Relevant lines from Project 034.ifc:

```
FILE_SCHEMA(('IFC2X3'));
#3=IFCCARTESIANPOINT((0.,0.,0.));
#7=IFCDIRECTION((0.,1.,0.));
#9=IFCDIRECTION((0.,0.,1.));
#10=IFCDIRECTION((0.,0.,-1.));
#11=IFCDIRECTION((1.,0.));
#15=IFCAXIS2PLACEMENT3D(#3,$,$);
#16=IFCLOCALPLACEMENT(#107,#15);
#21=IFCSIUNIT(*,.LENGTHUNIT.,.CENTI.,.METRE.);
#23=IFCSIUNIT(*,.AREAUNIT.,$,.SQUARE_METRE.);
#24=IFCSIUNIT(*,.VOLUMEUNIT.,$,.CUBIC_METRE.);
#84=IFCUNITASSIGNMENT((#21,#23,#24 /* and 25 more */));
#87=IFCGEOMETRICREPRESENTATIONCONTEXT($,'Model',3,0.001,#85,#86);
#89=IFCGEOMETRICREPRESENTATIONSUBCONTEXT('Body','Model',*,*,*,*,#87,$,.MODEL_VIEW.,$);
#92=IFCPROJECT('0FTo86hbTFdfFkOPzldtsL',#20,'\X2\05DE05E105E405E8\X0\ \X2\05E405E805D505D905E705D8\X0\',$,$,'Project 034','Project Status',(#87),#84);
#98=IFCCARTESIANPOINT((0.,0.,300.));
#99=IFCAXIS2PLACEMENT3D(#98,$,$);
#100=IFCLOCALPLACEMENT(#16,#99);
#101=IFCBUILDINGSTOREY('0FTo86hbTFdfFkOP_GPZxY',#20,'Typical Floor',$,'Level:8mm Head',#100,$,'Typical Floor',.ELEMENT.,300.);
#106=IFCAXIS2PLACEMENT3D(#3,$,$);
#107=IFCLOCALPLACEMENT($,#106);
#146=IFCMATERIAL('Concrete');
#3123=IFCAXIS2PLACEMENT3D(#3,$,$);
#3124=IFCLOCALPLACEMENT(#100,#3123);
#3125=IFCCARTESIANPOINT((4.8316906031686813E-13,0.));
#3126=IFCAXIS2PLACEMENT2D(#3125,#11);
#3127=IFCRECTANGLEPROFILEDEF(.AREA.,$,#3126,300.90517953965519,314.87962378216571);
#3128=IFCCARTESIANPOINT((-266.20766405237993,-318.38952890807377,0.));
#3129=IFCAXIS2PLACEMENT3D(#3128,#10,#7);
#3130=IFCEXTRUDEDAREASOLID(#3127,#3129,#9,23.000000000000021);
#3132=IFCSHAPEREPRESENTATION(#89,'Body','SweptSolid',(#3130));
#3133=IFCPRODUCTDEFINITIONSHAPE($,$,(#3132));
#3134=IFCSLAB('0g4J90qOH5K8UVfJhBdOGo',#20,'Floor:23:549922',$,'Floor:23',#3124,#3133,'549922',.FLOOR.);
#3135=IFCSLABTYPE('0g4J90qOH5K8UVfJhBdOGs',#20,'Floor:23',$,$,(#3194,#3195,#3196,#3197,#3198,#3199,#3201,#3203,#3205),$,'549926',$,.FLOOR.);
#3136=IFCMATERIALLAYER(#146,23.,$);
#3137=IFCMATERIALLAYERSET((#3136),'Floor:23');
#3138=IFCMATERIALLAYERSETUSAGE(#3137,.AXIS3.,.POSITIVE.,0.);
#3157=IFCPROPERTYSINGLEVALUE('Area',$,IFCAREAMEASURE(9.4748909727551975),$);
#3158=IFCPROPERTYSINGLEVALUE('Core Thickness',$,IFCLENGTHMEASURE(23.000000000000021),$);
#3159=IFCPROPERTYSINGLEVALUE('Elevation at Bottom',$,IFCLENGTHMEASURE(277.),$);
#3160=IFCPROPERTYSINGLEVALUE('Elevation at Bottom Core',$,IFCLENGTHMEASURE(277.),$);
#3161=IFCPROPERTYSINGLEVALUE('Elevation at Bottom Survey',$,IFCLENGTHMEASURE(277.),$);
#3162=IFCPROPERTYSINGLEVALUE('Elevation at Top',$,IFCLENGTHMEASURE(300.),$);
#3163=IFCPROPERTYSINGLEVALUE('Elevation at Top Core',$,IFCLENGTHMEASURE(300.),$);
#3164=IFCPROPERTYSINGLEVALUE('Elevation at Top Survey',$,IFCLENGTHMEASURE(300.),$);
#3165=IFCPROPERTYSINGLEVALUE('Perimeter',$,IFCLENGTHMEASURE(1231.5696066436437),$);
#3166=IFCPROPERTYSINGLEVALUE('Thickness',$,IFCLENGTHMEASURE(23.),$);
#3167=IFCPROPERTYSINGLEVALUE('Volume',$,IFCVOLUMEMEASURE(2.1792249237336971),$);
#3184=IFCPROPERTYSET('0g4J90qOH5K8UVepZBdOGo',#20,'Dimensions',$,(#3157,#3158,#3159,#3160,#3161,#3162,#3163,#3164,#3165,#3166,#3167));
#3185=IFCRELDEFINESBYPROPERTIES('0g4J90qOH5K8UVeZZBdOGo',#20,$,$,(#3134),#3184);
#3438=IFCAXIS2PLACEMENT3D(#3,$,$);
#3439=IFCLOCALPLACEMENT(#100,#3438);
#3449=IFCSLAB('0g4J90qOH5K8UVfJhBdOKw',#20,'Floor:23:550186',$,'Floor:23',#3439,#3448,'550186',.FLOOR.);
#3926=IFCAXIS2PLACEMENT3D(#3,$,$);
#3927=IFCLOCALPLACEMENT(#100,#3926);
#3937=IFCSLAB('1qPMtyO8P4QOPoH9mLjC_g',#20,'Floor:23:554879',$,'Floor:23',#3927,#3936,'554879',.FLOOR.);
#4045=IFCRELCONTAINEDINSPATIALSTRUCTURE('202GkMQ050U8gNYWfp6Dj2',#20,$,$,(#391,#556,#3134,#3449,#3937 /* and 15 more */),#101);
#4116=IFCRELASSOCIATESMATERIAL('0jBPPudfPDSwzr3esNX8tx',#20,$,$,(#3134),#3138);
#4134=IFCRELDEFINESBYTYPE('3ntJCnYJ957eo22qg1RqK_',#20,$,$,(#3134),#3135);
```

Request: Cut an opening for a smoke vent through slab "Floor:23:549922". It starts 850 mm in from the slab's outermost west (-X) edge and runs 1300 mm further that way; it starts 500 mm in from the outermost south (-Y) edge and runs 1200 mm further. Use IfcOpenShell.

```python
import numpy as np
import ifcopenshell
import ifcopenshell.api.feature
import ifcopenshell.api.geometry
import ifcopenshell.api.pset
import ifcopenshell.api.root
import ifcopenshell.geom
import ifcopenshell.util.element
import ifcopenshell.util.placement
import ifcopenshell.util.representation
import ifcopenshell.util.shape
import ifcopenshell.util.unit

model = ifcopenshell.open("Project 034.ifc")
unit_scale = ifcopenshell.util.unit.calculate_unit_scale(model)
area_scale = ifcopenshell.util.unit.calculate_unit_scale(model, "AREAUNIT")
volume_scale = ifcopenshell.util.unit.calculate_unit_scale(model, "VOLUMEUNIT")
settings = ifcopenshell.geom.settings()


def volume(element):
    """Net volume in cubic metres, openings subtracted."""
    shape = ifcopenshell.geom.create_shape(settings, element)
    return ifcopenshell.util.shape.get_volume(shape.geometry)


slab = model.by_id(3134)
before = volume(slab)

# Extent in the slab's own axes, in metres. The edges named are its -X and -Y sides.
slab_shape = ifcopenshell.geom.create_shape(settings, slab)
vertices = ifcopenshell.util.shape.get_vertices(slab_shape.geometry)
x_min, y_min, bottom = vertices.min(axis=0)
top = vertices[:, 2].max()

opening = ifcopenshell.api.root.create_entity(model, ifc_class="IfcOpeningElement", name="Smoke vent opening")
context = ifcopenshell.util.representation.get_context(model, "Model", "Body", "MODEL_VIEW")
width, depth = 1.3, 1.2
outline = [(0.0, 0.0), (width, 0.0), (width, depth), (0.0, depth), (0.0, 0.0)]
# Overshoot both faces by 50 mm so the cut is clean.
shape = ifcopenshell.api.geometry.add_slab_representation(
    model, context=context, depth=top - bottom + 0.1, polyline=outline
)
ifcopenshell.api.geometry.assign_representation(model, product=opening, representation=shape)

matrix = ifcopenshell.util.placement.get_local_placement(slab.ObjectPlacement)
matrix[:, 3] = matrix @ np.append(np.array([x_min + 0.85, y_min + 0.5, bottom - 0.05]) / unit_scale, 1.0)
ifcopenshell.api.geometry.edit_object_placement(model, product=opening, matrix=matrix, is_si=False)
ifcopenshell.api.feature.add_feature(model, feature=opening, element=slab)

after = volume(slab)

# Update the slab's stored quantities.
pset = model.by_id(ifcopenshell.util.element.get_pset(slab, "Dimensions", should_inherit=False)["id"])
ifcopenshell.api.pset.edit_pset(model, pset=pset, properties={
    "Area": model.create_entity("IfcAreaMeasure", after / (top - bottom) / area_scale),
    "Volume": model.create_entity("IfcVolumeMeasure", after / volume_scale),
})

print(f"slab volume {before:.3f} -> {after:.3f} m3")

model.write("Project 034_v2.ifc")
```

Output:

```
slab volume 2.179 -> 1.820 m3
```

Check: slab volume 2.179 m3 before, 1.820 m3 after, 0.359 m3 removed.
